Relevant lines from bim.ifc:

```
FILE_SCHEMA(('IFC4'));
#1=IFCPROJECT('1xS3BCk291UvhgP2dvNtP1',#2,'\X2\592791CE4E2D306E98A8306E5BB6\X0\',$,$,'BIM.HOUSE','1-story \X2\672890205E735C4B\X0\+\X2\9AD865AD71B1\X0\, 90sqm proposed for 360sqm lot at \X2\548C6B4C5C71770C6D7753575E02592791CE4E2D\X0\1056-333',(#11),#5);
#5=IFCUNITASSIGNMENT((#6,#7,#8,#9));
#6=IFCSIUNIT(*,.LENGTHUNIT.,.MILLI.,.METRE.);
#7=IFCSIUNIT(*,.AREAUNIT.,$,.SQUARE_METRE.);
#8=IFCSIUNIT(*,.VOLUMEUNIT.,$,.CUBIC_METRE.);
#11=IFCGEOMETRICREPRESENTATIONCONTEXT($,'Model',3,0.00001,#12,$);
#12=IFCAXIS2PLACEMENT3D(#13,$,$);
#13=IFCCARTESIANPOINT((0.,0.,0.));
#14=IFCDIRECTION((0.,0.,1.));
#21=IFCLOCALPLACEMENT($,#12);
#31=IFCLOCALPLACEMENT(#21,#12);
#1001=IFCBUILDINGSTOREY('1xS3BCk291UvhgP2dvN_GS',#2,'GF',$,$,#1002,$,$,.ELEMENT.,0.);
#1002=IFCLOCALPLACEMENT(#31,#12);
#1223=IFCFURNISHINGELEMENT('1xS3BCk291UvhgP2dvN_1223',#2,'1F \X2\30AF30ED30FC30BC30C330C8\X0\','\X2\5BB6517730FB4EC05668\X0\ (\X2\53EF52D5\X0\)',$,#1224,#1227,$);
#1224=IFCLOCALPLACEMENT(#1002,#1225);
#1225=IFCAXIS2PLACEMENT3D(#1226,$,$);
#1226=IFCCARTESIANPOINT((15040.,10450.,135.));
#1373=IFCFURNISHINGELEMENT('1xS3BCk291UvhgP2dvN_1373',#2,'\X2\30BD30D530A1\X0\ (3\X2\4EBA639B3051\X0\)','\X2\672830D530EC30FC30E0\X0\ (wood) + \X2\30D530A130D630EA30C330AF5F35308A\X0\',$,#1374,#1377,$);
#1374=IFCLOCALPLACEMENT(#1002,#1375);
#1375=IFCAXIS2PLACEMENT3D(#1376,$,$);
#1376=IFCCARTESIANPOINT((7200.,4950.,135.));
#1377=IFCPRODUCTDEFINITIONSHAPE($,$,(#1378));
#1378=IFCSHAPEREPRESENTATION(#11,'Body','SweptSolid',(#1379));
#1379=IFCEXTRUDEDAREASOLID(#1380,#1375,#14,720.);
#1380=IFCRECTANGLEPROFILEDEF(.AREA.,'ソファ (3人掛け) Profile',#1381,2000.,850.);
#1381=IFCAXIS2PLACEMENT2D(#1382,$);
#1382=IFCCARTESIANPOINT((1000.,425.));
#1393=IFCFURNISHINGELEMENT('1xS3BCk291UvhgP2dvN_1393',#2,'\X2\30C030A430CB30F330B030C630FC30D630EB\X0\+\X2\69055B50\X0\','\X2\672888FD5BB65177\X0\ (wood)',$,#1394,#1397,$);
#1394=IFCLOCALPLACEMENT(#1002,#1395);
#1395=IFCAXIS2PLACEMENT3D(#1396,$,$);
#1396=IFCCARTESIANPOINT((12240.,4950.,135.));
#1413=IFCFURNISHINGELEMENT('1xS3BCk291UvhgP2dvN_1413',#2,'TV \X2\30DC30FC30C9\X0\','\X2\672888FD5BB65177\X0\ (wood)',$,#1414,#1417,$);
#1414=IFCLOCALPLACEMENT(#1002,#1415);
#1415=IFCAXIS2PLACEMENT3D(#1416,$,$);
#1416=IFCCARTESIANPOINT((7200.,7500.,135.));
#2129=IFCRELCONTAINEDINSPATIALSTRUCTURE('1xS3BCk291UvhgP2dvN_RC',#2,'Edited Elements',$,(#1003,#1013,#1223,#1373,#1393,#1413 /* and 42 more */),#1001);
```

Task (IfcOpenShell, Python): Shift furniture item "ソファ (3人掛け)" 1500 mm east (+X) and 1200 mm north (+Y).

```python
import ifcopenshell
import ifcopenshell.api.geometry
import ifcopenshell.util.placement
import ifcopenshell.util.unit

model = ifcopenshell.open("bim.ifc")
unit_scale = ifcopenshell.util.unit.calculate_unit_scale(model)

item = model.by_guid("1xS3BCk291UvhgP2dvN_1373")
matrix = ifcopenshell.util.placement.get_local_placement(item.ObjectPlacement)
matrix[0, 3] += 1.5 / unit_scale
matrix[1, 3] += 1.2 / unit_scale
ifcopenshell.api.geometry.edit_object_placement(model, product=item, matrix=matrix, is_si=False)

print(ifcopenshell.util.placement.get_local_placement(item.ObjectPlacement).round(3) + 0.0)

model.write("bim_v2.ifc")
```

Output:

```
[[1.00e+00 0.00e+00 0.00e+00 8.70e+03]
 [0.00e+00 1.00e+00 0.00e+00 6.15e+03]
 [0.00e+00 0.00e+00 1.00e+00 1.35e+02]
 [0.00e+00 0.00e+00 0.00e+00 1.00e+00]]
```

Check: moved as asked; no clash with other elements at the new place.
